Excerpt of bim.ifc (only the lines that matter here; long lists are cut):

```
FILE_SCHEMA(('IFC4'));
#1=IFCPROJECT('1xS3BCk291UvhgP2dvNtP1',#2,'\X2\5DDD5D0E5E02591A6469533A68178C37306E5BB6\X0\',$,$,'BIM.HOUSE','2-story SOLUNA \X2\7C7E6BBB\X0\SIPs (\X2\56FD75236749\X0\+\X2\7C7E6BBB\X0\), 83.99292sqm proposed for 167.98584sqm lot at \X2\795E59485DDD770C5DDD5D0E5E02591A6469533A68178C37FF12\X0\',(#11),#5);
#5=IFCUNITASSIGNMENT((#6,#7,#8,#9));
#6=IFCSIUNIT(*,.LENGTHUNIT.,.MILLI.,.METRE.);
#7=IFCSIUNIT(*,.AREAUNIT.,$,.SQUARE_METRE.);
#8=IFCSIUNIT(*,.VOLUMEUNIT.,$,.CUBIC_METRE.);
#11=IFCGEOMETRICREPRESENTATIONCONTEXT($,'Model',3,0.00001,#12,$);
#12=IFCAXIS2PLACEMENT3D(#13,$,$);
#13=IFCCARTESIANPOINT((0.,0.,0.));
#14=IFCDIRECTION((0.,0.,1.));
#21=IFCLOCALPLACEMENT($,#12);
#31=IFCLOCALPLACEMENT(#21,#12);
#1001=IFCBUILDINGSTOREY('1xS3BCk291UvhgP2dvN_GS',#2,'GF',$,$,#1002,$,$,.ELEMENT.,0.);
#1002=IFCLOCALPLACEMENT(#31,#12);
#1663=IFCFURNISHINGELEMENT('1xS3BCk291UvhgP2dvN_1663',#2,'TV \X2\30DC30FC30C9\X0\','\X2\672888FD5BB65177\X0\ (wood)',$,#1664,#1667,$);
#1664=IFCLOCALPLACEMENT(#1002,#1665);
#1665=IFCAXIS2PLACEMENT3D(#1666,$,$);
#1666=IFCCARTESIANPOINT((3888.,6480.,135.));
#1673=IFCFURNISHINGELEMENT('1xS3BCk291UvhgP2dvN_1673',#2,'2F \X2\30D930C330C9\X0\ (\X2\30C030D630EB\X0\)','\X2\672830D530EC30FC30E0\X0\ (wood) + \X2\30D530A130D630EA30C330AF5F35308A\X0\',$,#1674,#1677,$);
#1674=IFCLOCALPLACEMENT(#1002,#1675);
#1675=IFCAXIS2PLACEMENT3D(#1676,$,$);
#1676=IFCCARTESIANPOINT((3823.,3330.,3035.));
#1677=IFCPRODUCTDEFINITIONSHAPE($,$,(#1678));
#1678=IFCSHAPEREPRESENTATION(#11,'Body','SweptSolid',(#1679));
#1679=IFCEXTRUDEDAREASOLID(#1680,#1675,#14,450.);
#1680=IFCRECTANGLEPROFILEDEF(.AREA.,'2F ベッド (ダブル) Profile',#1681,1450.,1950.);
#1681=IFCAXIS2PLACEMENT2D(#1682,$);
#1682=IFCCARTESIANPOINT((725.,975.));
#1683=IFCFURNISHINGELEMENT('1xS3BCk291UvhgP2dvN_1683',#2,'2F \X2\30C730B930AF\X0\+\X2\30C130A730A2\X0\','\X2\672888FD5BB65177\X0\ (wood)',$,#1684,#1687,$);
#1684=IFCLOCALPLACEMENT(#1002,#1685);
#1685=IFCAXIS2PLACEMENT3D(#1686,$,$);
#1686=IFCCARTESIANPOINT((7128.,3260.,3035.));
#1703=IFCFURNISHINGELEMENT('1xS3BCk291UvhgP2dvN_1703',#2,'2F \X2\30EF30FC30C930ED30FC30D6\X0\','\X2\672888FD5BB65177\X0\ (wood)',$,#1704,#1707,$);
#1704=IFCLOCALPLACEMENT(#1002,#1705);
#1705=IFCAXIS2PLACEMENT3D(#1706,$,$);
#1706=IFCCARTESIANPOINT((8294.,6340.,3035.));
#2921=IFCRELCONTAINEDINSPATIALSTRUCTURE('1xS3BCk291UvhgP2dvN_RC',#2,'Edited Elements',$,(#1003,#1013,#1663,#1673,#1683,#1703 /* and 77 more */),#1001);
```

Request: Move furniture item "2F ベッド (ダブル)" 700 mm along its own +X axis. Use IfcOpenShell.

```python
import ifcopenshell
import ifcopenshell.api.geometry
import ifcopenshell.util.placement

model = ifcopenshell.open("bim.ifc")

item = model.by_guid("1xS3BCk291UvhgP2dvN_1673")
matrix = ifcopenshell.util.placement.get_local_placement(item.ObjectPlacement)
matrix[:3, 3] += matrix[:3, 0] * 700.0
ifcopenshell.api.geometry.edit_object_placement(model, product=item, matrix=matrix, is_si=False)

print(ifcopenshell.util.placement.get_local_placement(item.ObjectPlacement).round(3) + 0.0)

model.write("bim_rev.ifc")
```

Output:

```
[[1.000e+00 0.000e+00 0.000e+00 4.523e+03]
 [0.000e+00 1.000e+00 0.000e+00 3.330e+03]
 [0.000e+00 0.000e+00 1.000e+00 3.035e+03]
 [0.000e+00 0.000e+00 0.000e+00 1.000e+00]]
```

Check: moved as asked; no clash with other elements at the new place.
